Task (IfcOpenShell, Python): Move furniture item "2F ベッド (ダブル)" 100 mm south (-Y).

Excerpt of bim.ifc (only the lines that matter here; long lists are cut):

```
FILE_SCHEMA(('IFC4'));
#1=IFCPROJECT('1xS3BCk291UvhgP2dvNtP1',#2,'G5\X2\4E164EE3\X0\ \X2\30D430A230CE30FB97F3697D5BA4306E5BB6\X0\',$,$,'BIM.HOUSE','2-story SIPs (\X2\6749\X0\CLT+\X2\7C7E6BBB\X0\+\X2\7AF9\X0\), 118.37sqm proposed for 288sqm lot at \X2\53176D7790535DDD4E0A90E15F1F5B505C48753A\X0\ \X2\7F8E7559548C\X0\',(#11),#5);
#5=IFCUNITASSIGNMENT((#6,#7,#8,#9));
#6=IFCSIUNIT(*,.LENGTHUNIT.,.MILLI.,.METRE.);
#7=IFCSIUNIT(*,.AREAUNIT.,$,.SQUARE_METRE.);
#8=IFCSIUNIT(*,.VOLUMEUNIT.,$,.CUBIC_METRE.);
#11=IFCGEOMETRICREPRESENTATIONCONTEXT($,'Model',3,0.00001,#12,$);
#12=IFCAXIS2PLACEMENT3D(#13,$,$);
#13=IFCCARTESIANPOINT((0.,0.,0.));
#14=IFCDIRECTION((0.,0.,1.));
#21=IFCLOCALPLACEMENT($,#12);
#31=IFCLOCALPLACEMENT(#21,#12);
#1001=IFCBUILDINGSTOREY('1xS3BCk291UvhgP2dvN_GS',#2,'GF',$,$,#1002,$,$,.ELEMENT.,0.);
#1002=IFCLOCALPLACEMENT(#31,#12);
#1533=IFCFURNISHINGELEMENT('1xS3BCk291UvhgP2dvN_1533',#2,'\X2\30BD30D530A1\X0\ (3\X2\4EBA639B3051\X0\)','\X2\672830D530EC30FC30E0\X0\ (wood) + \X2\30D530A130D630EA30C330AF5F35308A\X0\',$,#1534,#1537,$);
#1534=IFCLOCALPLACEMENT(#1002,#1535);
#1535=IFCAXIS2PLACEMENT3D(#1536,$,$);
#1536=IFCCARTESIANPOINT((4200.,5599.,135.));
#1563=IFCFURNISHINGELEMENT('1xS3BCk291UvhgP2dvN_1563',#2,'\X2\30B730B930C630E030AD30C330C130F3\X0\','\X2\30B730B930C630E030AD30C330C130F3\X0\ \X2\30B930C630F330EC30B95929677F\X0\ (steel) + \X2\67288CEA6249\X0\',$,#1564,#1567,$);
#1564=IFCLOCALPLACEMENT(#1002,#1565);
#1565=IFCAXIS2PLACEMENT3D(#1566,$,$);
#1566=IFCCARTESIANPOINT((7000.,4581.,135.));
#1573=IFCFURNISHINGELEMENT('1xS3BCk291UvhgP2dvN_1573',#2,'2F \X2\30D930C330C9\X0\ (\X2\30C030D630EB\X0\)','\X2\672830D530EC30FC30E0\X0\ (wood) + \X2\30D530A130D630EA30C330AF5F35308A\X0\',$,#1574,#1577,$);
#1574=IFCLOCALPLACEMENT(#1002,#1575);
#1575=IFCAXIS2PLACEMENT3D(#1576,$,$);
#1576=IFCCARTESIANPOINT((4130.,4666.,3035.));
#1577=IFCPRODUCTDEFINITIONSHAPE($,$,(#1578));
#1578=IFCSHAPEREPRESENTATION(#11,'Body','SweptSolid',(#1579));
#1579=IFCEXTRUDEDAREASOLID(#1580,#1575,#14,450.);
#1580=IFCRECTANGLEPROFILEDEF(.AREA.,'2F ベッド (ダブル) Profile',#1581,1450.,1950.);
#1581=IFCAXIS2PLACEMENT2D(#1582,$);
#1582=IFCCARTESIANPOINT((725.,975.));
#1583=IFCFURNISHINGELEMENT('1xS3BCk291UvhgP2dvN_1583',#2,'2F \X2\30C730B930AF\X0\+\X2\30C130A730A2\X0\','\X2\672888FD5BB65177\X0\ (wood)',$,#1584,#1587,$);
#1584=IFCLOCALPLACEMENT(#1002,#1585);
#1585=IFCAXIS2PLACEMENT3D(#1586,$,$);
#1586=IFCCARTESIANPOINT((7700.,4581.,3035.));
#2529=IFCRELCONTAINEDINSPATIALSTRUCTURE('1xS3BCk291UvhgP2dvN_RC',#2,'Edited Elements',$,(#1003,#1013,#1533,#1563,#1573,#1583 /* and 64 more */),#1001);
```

```python
import ifcopenshell
import ifcopenshell.api.geometry
import ifcopenshell.util.placement

model = ifcopenshell.open("bim.ifc")

item = model.by_guid("1xS3BCk291UvhgP2dvN_1573")
matrix = ifcopenshell.util.placement.get_local_placement(item.ObjectPlacement)
matrix[1, 3] -= 100.0
ifcopenshell.api.geometry.edit_object_placement(model, product=item, matrix=matrix, is_si=False)

print(ifcopenshell.util.placement.get_local_placement(item.ObjectPlacement).round(3) + 0.0)

model.write("bim_updated.ifc")
```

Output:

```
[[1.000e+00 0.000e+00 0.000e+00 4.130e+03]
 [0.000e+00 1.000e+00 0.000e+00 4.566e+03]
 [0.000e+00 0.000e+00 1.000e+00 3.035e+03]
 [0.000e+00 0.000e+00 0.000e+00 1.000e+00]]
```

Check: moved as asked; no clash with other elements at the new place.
